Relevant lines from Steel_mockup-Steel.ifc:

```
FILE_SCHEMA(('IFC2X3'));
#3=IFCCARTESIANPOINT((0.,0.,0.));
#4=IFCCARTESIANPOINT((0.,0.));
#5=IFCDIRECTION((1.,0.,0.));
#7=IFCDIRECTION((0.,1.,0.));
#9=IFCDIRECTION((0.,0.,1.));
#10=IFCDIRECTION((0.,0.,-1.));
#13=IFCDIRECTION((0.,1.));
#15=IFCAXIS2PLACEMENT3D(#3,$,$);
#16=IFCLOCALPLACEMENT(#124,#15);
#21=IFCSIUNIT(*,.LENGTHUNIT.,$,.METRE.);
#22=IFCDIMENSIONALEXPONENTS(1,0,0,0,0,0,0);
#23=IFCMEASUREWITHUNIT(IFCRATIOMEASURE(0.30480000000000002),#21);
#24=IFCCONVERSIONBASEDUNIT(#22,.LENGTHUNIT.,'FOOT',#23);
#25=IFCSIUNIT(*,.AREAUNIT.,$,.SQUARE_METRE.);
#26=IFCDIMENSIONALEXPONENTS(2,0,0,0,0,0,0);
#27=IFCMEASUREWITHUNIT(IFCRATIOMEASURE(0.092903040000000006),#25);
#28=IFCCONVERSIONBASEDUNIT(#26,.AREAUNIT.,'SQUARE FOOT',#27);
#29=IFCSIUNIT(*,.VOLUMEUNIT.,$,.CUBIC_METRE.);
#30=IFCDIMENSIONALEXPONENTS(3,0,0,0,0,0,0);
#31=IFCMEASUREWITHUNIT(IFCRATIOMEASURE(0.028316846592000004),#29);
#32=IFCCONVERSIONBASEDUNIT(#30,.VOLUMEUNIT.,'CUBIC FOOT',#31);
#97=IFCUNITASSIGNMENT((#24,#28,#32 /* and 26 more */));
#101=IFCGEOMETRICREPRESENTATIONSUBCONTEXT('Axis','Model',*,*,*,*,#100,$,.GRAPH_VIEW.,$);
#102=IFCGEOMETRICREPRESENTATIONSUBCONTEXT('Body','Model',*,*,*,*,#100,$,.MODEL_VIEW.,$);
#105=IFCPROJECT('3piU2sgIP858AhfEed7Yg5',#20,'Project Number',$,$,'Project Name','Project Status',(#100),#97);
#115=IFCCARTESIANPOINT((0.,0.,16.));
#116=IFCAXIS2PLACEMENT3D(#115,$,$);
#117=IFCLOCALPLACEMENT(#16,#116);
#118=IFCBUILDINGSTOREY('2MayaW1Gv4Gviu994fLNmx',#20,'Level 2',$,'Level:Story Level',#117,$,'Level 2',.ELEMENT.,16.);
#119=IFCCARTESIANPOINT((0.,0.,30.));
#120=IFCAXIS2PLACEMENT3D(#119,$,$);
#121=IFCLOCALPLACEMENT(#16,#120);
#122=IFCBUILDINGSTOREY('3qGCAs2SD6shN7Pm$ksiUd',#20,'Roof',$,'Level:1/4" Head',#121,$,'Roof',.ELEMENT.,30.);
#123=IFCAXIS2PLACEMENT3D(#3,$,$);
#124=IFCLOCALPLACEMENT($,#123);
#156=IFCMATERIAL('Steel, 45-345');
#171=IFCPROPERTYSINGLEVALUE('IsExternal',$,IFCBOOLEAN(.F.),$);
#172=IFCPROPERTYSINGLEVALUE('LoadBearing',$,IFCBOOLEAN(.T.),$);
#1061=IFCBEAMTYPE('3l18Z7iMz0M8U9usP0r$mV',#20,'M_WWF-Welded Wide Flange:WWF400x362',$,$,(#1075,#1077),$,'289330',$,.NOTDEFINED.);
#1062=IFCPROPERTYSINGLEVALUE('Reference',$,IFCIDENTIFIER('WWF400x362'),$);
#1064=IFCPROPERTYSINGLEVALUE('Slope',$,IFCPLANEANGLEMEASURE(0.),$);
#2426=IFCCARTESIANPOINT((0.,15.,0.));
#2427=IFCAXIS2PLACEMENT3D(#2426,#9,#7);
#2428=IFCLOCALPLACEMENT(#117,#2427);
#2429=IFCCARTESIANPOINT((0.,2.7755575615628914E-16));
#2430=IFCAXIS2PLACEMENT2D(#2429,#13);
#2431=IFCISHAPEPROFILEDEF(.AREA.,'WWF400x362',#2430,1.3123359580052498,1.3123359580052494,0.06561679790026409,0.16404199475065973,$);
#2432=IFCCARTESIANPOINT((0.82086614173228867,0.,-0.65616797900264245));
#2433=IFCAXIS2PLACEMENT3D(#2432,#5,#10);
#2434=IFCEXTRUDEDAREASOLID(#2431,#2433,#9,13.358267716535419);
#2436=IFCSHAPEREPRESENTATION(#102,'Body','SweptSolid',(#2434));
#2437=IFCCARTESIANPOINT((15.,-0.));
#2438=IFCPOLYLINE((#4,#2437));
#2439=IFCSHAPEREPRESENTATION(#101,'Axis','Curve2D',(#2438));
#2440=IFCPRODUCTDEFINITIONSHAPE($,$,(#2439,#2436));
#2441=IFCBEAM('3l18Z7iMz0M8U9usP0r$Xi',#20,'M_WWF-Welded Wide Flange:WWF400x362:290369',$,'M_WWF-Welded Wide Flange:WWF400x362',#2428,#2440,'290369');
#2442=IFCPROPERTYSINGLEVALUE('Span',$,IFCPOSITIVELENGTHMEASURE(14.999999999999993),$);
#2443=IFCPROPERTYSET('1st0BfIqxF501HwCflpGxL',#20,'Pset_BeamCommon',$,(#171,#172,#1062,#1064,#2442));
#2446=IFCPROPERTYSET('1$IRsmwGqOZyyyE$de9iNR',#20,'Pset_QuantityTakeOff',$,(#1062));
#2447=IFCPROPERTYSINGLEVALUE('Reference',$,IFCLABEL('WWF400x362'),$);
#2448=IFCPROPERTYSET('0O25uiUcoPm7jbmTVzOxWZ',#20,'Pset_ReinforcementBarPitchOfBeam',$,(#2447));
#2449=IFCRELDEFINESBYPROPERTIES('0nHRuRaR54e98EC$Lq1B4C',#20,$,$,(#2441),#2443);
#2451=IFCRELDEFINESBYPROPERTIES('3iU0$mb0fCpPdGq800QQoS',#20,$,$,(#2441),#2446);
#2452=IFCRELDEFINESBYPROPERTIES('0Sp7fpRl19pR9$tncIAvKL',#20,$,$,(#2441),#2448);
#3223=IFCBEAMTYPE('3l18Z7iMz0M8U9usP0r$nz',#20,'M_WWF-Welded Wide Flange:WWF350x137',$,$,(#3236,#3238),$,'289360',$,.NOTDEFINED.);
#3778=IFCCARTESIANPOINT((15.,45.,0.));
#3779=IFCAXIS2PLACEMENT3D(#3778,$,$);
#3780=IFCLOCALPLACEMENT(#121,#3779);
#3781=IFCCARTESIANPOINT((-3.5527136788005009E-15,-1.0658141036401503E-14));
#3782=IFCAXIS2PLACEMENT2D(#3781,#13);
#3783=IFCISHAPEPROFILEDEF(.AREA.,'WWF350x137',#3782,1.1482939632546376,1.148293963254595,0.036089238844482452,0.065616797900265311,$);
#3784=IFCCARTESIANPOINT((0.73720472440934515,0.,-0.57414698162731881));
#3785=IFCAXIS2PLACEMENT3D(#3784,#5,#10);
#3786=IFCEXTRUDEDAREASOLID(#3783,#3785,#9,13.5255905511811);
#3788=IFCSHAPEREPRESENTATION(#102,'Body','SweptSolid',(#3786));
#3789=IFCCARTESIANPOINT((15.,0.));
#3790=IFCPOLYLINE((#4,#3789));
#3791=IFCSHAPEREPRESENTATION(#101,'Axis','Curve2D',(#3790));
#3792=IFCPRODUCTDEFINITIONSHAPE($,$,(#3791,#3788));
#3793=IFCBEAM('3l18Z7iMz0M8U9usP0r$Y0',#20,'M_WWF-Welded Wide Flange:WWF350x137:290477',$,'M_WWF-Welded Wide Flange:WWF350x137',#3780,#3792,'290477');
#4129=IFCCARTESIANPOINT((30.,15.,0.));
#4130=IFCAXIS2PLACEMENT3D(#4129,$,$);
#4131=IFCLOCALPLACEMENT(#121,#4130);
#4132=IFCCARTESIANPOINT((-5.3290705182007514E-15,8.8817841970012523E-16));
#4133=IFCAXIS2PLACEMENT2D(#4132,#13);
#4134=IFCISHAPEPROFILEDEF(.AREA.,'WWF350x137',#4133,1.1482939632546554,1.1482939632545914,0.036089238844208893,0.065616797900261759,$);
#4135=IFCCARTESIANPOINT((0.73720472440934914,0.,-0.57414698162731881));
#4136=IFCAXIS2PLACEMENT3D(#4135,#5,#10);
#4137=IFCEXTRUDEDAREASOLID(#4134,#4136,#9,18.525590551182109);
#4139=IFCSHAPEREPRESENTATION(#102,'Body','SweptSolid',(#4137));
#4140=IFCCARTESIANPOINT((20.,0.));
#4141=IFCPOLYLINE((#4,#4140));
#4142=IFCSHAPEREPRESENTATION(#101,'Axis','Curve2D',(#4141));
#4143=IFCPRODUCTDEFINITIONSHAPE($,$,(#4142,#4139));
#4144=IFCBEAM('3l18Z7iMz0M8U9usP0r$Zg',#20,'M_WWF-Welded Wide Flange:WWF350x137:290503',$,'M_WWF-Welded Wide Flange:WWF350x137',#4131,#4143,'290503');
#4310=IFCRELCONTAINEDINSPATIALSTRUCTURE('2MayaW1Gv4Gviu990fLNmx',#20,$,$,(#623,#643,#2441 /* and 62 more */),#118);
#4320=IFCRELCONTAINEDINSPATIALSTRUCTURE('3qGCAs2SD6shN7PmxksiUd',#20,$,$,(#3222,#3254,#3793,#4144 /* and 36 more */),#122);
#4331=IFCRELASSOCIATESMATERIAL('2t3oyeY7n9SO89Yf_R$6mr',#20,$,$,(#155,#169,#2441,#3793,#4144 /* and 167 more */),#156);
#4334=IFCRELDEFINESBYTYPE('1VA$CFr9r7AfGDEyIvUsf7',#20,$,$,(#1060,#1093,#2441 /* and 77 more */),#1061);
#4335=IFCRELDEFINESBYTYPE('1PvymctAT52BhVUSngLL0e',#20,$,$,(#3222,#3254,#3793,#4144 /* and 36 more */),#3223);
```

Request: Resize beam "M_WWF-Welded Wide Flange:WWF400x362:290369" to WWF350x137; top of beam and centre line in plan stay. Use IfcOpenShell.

```python
import ifcopenshell
import ifcopenshell.api.pset
import ifcopenshell.api.type
import ifcopenshell.util.element
import ifcopenshell.util.representation

model = ifcopenshell.open("Steel_mockup-Steel.ifc")

member = model.by_guid("3l18Z7iMz0M8U9usP0r$Xi")
source = next(p for p in model.by_type("IfcIShapeProfileDef") if p.ProfileName == "WWF350x137")

body = ifcopenshell.util.representation.get_representation(member, "Model", "Body")
solid = body.Items[0]
old_profile = solid.SweptArea

# Copy the section's sizes but keep this member's own profile position.
profile = ifcopenshell.util.element.copy(model, source)
# Profiles are centred, so shift by half the change in depth to hold the top.
shift = (old_profile.OverallDepth - profile.OverallDepth) / 2
x, y = old_profile.Position.Location.Coordinates
up = (-1.0, 0.0)  # upwards, in the solid's own plane
location = model.createIfcCartesianPoint((x + up[0] * shift, y + up[1] * shift))
profile.Position = model.createIfcAxis2Placement2D(location, old_profile.Position.RefDirection)
solid.SweptArea = profile
if not model.get_total_inverses(old_profile):
    ifcopenshell.util.element.remove_deep2(model, old_profile)

new_type = model.by_guid("3l18Z7iMz0M8U9usP0r$nz")
ifcopenshell.api.type.assign_type(
    model, related_objects=[member], relating_type=new_type, should_map_representations=False
)
member.Name = member.Name.replace("WWF400x362", "WWF350x137")
member.ObjectType = "M_WWF-Welded Wide Flange:WWF350x137"
pset = model.by_id(ifcopenshell.util.element.get_pset(member, "Pset_BeamCommon", should_inherit=False)["id"])
ifcopenshell.api.pset.edit_pset(model, pset=pset, properties={"Reference": "WWF350x137"})
pset = model.by_id(ifcopenshell.util.element.get_pset(member, "Pset_QuantityTakeOff", should_inherit=False)["id"])
ifcopenshell.api.pset.edit_pset(model, pset=pset, properties={"Reference": "WWF350x137"})
pset = model.by_id(ifcopenshell.util.element.get_pset(member, "Pset_ReinforcementBarPitchOfBeam", should_inherit=False)["id"])
ifcopenshell.api.pset.edit_pset(model, pset=pset, properties={"Reference": "WWF350x137"})

print(solid.SweptArea)

model.write("Steel_mockup-Steel_v2.ifc")
```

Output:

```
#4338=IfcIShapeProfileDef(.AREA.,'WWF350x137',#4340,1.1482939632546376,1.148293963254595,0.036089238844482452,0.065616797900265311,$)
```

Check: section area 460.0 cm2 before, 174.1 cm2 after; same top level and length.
